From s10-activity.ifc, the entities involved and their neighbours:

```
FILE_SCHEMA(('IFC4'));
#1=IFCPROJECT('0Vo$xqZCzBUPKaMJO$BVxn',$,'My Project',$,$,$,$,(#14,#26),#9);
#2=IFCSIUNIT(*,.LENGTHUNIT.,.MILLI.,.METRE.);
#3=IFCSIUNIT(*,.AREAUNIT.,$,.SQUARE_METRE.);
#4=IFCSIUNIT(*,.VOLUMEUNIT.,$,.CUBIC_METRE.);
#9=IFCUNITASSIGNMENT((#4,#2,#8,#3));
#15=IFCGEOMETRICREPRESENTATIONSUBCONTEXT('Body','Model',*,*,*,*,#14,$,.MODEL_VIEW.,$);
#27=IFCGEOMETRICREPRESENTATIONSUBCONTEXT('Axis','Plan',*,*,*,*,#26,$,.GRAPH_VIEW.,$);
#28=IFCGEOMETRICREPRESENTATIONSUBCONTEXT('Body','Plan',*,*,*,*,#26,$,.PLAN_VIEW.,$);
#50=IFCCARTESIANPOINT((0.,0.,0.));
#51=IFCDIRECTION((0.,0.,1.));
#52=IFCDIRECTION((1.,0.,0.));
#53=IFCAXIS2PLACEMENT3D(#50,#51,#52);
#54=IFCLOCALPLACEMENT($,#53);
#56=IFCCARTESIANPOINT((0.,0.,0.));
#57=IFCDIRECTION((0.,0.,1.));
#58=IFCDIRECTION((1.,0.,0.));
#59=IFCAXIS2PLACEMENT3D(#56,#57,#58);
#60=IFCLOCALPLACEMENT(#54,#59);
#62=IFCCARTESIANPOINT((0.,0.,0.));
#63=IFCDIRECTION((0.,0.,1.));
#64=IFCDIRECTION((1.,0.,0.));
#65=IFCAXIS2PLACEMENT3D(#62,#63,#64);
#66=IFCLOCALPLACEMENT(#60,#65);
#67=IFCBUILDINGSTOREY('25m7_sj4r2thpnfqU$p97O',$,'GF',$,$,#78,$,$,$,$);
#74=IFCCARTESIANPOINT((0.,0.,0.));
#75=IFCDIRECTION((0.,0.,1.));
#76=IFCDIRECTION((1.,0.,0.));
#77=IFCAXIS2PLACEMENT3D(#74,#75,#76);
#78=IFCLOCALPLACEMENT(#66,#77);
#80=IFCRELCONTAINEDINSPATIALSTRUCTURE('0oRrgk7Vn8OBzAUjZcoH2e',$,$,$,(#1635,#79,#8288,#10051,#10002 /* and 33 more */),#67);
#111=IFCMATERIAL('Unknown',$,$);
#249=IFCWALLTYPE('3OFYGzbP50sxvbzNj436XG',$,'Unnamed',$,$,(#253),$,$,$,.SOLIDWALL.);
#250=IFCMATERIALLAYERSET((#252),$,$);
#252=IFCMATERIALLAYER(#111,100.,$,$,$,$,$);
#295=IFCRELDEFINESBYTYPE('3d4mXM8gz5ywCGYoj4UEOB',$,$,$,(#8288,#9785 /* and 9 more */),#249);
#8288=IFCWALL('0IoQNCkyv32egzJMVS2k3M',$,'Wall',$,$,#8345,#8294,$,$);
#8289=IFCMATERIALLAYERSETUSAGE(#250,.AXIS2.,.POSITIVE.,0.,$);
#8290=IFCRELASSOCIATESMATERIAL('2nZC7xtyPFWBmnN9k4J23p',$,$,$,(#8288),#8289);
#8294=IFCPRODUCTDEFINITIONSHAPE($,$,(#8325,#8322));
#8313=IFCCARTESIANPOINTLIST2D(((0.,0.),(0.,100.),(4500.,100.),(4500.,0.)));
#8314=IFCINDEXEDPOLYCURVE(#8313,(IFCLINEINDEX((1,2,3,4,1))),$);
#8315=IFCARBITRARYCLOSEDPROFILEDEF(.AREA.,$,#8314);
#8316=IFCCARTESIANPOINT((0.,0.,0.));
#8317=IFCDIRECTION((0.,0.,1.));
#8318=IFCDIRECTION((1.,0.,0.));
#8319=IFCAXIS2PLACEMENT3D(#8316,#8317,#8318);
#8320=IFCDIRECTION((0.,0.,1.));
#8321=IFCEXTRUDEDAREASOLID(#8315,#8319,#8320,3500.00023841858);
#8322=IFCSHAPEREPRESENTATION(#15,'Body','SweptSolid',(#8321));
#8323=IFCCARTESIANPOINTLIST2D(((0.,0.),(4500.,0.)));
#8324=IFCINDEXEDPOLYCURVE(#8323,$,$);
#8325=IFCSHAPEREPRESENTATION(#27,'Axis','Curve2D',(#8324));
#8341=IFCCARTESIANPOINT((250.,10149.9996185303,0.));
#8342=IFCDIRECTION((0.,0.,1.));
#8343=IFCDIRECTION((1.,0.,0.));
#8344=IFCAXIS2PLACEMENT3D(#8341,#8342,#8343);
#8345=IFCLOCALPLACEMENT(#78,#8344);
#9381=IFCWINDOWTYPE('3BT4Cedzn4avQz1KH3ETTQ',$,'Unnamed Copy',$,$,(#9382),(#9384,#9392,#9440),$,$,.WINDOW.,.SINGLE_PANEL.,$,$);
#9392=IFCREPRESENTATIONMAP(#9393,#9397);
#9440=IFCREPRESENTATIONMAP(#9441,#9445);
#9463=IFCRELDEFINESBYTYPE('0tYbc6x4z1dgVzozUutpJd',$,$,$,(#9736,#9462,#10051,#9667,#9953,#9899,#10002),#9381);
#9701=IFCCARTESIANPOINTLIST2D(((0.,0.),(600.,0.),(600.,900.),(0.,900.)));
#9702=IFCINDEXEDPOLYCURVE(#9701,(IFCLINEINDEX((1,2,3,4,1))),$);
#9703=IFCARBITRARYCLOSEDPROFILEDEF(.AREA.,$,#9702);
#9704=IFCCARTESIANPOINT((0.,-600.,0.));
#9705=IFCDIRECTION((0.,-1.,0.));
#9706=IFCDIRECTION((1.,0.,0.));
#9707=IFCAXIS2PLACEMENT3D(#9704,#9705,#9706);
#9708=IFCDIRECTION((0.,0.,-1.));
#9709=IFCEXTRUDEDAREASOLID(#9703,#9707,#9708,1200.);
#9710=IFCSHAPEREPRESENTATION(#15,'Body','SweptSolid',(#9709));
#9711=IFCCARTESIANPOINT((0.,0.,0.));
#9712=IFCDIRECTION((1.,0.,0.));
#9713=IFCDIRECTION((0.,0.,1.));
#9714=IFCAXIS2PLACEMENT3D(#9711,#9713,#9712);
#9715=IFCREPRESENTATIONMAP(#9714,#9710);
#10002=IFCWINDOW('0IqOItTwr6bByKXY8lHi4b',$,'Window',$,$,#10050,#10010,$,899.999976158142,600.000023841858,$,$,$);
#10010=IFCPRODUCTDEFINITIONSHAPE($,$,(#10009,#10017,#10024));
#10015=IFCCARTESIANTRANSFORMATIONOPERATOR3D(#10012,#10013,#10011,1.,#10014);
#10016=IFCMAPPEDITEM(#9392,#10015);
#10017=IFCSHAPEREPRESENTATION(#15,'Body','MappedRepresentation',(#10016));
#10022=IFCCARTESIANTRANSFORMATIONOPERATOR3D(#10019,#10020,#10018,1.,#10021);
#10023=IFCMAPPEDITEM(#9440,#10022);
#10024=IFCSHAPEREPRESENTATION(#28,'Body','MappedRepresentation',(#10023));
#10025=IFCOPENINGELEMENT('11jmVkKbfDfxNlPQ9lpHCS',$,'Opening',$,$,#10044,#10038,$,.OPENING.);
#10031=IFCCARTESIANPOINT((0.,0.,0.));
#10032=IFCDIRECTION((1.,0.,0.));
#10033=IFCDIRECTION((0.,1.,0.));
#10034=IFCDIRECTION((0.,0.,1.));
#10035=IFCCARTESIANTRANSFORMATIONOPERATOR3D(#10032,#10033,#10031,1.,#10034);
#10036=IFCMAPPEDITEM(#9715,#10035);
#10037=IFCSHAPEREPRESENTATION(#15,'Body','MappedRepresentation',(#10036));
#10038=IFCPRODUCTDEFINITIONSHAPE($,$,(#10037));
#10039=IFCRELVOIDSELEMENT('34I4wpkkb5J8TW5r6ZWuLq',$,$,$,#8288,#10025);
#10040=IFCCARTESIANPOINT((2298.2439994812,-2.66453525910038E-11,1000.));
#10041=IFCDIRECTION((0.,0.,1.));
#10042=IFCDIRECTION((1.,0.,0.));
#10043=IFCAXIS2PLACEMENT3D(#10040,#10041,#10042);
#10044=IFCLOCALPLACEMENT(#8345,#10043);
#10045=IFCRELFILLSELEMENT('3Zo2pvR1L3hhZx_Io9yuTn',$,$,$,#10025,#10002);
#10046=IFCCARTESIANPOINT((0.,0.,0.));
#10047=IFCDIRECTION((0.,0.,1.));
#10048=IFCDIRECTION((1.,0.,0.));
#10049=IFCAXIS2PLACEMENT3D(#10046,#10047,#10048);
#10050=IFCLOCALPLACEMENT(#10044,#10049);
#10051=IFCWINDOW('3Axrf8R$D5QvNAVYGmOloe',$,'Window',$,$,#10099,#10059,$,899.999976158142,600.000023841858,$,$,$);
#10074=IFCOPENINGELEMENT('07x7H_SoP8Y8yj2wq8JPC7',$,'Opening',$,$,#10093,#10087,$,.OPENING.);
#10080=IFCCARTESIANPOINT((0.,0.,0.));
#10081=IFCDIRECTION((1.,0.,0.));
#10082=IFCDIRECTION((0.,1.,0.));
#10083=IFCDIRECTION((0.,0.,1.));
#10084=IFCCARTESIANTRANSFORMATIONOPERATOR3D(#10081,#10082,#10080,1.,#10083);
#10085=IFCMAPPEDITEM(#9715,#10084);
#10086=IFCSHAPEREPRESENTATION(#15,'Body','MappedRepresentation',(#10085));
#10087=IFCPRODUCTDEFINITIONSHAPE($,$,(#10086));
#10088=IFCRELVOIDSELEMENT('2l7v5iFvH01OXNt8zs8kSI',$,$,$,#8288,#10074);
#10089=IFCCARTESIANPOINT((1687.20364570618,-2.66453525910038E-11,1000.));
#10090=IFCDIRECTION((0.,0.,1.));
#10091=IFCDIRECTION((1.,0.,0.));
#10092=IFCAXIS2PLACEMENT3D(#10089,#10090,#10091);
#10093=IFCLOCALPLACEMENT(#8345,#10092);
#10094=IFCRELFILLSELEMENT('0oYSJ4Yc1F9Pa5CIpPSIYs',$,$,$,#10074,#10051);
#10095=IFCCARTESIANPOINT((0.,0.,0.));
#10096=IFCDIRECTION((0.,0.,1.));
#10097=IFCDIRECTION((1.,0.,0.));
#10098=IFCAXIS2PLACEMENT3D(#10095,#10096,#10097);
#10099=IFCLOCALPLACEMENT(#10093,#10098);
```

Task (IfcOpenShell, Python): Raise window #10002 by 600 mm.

```python
import numpy as np
import ifcopenshell
import ifcopenshell.api.geometry
import ifcopenshell.util.placement
import ifcopenshell.util.unit

model = ifcopenshell.open("s10-activity.ifc")
unit_scale = ifcopenshell.util.unit.calculate_unit_scale(model)

window = model.by_id(10002)
opening = window.FillsVoids[0].RelatingOpeningElement
dz = 0.6 / unit_scale

shift = np.array([0.0, 0.0, dz])
# The window is placed relative to its opening, so it follows when the opening moves.
matrix = ifcopenshell.util.placement.get_local_placement(opening.ObjectPlacement)
matrix[:3, 3] += shift
ifcopenshell.api.geometry.edit_object_placement(
    model, product=opening, matrix=matrix, is_si=False, should_transform_children=True
)

print(f"moved by {dz * unit_scale:+.3f} m")

model.write("s10-activity_edited.ifc")
```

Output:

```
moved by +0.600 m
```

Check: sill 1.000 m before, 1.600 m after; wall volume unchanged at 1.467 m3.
